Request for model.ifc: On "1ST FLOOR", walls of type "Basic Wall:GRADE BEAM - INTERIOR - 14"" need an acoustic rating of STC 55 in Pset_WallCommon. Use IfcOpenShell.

First a look at what the model holds.

```python
import ifcopenshell
import ifcopenshell.util.element

model = ifcopenshell.open("model.ifc")
print(model.schema)
storey = next(s for s in model.by_type("IfcBuildingStorey") if s.Name == "1ST FLOOR")
walls = [e for e in ifcopenshell.util.element.get_decomposition(storey) if e.is_a("IfcWall")]
seen = {}
for e in walls:
    element_type = ifcopenshell.util.element.get_type(e)
    key = (element_type.Name if element_type != e and element_type else None, ifcopenshell.util.element.get_pset(e, "Pset_WallCommon", "AcousticRating"))
    seen[key] = seen.get(key, 0) + 1
for (name, value), count in sorted(seen.items(), key=str):
    print(count, "x", name, "|", value)
```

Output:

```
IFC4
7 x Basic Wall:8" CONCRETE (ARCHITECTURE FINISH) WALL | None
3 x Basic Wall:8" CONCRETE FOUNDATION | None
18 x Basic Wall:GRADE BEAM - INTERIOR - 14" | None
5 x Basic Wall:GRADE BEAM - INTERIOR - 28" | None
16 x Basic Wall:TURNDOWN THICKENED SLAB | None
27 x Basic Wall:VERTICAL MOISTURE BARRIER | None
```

```python
import ifcopenshell
import ifcopenshell.api.pset
import ifcopenshell.util.element

model = ifcopenshell.open("model.ifc")

storey = next(s for s in model.by_type("IfcBuildingStorey") if s.Name == "1ST FLOOR")
walls = [e for e in ifcopenshell.util.element.get_decomposition(storey) if e.is_a("IfcWall")]

count = 0
for e in walls:
    element_type = ifcopenshell.util.element.get_type(e)
    if element_type in (None, e) or element_type.Name != 'Basic Wall:GRADE BEAM - INTERIOR - 14"':
        continue
    # add_pset returns the element's existing set when there is one.
    pset = ifcopenshell.api.pset.add_pset(model, product=e, name="Pset_WallCommon")
    ifcopenshell.api.pset.edit_pset(model, pset=pset, properties={"AcousticRating": "STC 55"})
    count += 1

print(count, "walls updated")

model.write("model_v2.ifc")
```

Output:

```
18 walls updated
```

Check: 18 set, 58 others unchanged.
